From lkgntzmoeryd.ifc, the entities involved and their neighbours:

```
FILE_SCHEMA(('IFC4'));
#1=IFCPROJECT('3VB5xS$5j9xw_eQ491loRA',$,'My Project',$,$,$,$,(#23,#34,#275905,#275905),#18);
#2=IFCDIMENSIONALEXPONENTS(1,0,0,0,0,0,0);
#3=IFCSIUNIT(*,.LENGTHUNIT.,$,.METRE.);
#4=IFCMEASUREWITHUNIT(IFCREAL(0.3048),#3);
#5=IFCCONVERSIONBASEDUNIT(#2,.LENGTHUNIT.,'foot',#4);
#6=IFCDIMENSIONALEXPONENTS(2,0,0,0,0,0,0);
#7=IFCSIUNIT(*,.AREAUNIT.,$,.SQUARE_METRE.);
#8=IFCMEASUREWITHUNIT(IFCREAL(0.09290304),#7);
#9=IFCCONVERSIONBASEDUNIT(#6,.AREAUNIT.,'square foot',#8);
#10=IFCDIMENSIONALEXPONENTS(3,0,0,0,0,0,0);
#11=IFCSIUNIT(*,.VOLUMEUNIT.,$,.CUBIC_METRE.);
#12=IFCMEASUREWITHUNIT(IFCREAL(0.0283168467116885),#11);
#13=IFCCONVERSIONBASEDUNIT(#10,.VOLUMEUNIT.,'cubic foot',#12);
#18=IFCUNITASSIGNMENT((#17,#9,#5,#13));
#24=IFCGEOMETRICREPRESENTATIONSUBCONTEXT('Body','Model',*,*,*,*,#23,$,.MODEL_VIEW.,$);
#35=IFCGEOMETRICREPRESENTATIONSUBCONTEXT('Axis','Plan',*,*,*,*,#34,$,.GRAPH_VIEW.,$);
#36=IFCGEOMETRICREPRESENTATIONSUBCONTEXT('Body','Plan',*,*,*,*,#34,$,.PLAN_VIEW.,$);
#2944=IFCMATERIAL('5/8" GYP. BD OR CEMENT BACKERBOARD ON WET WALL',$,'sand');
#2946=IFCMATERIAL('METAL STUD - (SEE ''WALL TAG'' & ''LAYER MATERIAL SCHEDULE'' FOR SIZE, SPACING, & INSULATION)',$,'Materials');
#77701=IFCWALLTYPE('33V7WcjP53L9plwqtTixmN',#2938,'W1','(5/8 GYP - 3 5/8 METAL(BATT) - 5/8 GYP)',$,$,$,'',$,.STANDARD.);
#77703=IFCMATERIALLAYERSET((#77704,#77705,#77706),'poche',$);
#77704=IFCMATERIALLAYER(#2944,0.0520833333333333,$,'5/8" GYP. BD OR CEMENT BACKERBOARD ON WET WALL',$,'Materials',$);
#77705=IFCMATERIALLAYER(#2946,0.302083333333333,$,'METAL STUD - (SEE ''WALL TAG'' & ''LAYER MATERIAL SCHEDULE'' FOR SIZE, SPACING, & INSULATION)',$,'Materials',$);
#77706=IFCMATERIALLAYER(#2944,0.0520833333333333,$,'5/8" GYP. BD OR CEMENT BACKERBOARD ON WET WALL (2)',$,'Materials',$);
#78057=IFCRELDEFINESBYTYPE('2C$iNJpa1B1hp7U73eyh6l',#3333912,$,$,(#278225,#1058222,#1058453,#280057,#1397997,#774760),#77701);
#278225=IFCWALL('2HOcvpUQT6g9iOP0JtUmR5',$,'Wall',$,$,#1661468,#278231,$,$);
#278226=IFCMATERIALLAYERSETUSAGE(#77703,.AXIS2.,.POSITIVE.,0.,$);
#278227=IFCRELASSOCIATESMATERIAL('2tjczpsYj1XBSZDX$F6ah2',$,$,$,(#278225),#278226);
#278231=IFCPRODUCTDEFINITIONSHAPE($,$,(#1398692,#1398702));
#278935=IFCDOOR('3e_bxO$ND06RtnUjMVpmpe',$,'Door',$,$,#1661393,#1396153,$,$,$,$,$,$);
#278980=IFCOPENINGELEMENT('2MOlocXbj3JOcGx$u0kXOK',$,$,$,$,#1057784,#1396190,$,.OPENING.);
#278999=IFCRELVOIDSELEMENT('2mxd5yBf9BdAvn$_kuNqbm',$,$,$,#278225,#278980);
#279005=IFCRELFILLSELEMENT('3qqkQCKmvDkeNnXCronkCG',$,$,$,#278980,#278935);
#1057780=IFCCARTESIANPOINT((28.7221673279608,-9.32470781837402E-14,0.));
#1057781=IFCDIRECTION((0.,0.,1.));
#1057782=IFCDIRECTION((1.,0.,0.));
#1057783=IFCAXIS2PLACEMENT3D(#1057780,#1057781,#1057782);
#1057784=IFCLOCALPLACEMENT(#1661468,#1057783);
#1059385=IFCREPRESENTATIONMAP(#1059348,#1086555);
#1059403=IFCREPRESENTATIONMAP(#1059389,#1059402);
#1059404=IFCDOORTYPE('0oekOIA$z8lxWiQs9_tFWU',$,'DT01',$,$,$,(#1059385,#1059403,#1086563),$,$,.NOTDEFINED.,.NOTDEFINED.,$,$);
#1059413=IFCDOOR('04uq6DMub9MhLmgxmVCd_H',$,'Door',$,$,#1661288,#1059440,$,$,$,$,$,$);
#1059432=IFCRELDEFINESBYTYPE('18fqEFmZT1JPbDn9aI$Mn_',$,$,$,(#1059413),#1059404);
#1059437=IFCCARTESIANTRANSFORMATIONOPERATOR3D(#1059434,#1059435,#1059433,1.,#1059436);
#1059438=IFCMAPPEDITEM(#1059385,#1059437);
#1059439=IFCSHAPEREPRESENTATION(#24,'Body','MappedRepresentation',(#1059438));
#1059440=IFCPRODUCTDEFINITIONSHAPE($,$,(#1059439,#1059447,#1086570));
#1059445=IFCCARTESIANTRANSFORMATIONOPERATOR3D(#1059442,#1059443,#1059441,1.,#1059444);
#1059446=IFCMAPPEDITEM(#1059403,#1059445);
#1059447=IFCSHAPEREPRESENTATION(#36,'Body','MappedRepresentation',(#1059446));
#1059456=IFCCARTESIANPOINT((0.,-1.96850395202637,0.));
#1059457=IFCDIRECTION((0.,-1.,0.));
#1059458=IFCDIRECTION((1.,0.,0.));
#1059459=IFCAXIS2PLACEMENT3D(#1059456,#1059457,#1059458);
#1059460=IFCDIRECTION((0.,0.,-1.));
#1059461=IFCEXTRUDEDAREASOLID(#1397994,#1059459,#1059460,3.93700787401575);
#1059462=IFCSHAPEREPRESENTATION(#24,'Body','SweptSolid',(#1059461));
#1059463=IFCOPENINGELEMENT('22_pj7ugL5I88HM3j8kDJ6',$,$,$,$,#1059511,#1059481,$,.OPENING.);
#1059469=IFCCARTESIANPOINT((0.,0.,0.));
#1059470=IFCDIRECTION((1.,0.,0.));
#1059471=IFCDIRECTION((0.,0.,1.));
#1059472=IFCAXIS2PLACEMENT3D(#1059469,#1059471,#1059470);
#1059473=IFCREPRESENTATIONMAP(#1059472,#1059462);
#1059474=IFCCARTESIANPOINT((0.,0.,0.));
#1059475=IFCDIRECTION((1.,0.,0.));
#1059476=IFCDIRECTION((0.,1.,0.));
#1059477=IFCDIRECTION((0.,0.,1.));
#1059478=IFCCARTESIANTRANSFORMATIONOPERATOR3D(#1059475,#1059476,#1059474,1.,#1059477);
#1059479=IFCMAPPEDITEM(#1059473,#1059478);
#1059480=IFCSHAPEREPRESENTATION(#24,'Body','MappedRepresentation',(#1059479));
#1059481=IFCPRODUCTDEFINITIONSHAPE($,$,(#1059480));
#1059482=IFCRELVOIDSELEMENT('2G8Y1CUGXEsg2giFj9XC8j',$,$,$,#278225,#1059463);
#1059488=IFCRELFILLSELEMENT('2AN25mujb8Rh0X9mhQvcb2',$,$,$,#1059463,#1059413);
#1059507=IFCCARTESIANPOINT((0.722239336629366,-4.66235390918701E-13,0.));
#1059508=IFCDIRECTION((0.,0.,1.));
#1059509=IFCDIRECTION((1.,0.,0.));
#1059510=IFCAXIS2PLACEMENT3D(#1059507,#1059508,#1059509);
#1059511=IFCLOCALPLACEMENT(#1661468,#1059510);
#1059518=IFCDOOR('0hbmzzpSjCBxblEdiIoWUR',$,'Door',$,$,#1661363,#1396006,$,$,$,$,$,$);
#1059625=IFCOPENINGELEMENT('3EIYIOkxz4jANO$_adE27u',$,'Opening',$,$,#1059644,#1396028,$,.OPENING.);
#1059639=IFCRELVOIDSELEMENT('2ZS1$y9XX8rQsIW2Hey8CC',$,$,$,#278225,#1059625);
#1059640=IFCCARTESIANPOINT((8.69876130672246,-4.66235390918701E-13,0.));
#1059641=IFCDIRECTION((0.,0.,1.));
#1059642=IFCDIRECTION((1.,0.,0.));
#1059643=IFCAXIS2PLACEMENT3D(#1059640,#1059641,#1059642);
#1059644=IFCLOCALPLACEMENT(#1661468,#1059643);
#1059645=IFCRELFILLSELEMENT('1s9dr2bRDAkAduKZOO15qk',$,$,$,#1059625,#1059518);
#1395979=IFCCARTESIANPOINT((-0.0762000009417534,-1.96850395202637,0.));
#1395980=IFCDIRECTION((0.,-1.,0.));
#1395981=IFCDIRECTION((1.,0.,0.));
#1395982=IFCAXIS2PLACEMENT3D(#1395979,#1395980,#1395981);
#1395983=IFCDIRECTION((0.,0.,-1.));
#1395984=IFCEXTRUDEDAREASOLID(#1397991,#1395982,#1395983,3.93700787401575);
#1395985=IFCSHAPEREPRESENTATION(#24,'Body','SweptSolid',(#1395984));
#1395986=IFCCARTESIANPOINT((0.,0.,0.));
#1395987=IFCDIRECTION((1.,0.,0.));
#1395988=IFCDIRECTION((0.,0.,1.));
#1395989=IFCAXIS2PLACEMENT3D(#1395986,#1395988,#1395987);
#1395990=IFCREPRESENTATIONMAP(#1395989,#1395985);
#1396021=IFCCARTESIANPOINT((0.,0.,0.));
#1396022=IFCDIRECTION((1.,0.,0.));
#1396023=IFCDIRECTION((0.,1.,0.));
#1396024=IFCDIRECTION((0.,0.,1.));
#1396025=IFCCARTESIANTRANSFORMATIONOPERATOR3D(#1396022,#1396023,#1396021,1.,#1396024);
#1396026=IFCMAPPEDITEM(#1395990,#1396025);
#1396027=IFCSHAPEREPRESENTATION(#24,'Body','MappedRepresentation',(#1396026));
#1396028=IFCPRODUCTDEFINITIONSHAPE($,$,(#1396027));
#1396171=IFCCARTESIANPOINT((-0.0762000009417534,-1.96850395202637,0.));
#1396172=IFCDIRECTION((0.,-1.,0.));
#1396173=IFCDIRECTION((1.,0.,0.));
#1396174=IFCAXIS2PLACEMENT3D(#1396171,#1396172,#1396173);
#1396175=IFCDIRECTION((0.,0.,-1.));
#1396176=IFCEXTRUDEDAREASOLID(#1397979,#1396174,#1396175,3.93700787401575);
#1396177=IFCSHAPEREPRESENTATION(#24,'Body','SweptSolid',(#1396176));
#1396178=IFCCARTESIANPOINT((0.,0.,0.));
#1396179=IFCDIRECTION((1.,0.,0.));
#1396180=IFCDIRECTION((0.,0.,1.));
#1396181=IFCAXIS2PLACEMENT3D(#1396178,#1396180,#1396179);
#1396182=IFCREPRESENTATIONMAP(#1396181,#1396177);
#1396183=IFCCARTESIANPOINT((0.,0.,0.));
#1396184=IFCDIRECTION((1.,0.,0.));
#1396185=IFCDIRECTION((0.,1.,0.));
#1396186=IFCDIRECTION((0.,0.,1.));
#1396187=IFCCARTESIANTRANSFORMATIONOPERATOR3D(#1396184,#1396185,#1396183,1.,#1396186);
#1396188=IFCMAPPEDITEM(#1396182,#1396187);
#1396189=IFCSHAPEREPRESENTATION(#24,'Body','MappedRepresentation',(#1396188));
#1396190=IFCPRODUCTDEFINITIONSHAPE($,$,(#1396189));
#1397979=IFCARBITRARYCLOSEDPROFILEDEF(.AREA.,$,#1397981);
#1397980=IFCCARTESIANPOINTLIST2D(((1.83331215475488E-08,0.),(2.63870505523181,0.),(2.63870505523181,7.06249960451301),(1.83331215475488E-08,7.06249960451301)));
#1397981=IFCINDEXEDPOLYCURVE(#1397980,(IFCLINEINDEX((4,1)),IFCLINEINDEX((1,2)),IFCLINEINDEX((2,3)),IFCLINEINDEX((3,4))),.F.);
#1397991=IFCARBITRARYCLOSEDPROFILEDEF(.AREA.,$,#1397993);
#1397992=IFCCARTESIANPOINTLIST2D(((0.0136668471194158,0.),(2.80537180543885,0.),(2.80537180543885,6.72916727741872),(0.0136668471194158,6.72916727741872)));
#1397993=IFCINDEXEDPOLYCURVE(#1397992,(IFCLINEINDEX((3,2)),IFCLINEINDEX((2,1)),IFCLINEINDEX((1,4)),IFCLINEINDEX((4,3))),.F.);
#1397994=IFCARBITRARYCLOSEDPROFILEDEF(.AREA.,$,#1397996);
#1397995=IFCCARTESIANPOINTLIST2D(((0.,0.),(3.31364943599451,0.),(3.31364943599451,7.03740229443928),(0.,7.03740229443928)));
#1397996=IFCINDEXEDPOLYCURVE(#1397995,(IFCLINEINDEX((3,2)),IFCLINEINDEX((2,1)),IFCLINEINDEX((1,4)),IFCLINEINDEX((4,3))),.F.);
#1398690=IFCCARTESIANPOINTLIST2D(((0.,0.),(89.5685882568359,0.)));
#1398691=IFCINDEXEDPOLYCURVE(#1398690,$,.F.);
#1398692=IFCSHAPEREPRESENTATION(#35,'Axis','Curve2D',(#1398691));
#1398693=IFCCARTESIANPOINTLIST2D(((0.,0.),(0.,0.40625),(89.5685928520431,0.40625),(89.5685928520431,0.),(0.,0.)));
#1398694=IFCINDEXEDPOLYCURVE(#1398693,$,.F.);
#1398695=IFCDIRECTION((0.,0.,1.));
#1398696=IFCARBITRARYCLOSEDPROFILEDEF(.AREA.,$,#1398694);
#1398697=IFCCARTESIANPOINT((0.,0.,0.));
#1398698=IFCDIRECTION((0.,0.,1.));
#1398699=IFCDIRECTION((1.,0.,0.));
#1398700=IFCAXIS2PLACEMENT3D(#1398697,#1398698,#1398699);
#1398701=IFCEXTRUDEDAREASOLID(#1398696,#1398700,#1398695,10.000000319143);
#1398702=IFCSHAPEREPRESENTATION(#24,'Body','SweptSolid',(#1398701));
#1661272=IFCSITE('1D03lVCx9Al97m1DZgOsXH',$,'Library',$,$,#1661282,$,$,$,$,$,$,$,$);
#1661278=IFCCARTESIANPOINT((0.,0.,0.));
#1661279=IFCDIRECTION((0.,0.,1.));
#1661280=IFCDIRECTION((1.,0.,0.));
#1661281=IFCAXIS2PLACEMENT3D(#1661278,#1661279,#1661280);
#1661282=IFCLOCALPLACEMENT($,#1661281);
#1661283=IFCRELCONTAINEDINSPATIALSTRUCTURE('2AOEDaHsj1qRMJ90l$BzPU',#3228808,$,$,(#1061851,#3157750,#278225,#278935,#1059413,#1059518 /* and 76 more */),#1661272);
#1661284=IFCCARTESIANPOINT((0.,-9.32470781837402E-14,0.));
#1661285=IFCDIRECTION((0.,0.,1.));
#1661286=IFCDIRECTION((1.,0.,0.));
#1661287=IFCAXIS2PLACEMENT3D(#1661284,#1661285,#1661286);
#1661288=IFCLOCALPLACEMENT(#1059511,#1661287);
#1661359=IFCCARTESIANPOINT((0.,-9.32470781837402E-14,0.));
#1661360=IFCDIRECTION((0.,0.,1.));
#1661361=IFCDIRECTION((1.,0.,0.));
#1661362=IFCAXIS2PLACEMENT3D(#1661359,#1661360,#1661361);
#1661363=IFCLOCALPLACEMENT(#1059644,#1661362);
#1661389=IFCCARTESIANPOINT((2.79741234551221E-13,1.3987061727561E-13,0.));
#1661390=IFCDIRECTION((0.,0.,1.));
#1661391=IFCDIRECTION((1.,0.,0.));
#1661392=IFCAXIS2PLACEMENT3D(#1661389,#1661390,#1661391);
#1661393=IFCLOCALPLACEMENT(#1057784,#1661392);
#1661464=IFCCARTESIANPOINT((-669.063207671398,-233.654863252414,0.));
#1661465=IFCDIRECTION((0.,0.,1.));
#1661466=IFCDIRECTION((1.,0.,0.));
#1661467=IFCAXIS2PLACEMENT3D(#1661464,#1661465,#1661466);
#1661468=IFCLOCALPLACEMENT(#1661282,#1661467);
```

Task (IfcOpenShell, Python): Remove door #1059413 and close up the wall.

```python
import ifcopenshell
import ifcopenshell.api.feature
import ifcopenshell.api.root
import ifcopenshell.geom
import ifcopenshell.util.shape

model = ifcopenshell.open("lkgntzmoeryd.ifc")
settings = ifcopenshell.geom.settings()


def volume(element):
    """Net volume in cubic metres, openings subtracted."""
    shape = ifcopenshell.geom.create_shape(settings, element)
    return ifcopenshell.util.shape.get_volume(shape.geometry)


door = model.by_guid("04uq6DMub9MhLmgxmVCd_H")
opening = door.FillsVoids[0].RelatingOpeningElement
wall = opening.VoidsElements[0].RelatingBuildingElement
before = volume(wall)

ifcopenshell.api.root.remove_product(model, product=door)
ifcopenshell.api.feature.remove_feature(model, feature=opening)

after = volume(wall)

print(f"wall volume {before:.3f} -> {after:.3f} m3")

model.write("lkgntzmoeryd_edited.ifc")
```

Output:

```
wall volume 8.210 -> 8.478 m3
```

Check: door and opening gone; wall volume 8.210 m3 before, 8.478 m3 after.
